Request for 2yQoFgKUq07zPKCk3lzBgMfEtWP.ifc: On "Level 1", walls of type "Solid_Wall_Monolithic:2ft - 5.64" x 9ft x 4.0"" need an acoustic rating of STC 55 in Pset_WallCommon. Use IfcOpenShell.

First a look at what the model holds.

```python
import ifcopenshell
import ifcopenshell.util.element

model = ifcopenshell.open("2yQoFgKUq07zPKCk3lzBgMfEtWP.ifc")
print(model.schema)
storey = next(s for s in model.by_type("IfcBuildingStorey") if s.Name == "Level 1")
walls = [e for e in ifcopenshell.util.element.get_decomposition(storey) if e.is_a("IfcWall")]
seen = {}
for e in walls:
    element_type = ifcopenshell.util.element.get_type(e)
    key = (element_type.Name if element_type != e and element_type else None, ifcopenshell.util.element.get_pset(e, "Pset_WallCommon", "AcousticRating"))
    seen[key] = seen.get(key, 0) + 1
for (name, value), count in sorted(seen.items(), key=str):
    print(count, "x", name, "|", value)
```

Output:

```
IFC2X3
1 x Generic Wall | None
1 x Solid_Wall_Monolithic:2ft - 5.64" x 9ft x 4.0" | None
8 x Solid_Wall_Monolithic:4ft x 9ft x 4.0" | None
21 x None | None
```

```python
import ifcopenshell
import ifcopenshell.api.pset
import ifcopenshell.util.element

model = ifcopenshell.open("2yQoFgKUq07zPKCk3lzBgMfEtWP.ifc")

storey = next(s for s in model.by_type("IfcBuildingStorey") if s.Name == "Level 1")
walls = [e for e in ifcopenshell.util.element.get_decomposition(storey) if e.is_a("IfcWall")]

count = 0
for e in walls:
    element_type = ifcopenshell.util.element.get_type(e)
    if element_type in (None, e) or element_type.Name != 'Solid_Wall_Monolithic:2ft - 5.64" x 9ft x 4.0"':
        continue
    # add_pset returns the element's existing set when there is one.
    pset = ifcopenshell.api.pset.add_pset(model, product=e, name="Pset_WallCommon")
    ifcopenshell.api.pset.edit_pset(model, pset=pset, properties={"AcousticRating": "STC 55"})
    count += 1

print(count, "walls updated")

model.write("2yQoFgKUq07zPKCk3lzBgMfEtWP_v2.ifc")
```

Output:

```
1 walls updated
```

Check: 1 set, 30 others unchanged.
